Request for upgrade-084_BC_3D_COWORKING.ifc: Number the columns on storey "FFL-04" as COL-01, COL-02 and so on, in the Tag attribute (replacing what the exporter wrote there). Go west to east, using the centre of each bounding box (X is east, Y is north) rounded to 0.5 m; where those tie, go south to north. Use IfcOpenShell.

First a look at what the model holds.

```python
import ifcopenshell
import ifcopenshell.util.element
import ifcopenshell.util.placement

model = ifcopenshell.open("upgrade-084_BC_3D_COWORKING.ifc")
print(model.schema)
storey = next(s for s in model.by_type("IfcBuildingStorey") if s.Name == "FFL-04")
columns = [e for e in ifcopenshell.util.element.get_decomposition(storey) if e.is_a("IfcColumn")]
for e in sorted(columns, key=lambda e: e.id()):
    origin = ifcopenshell.util.placement.get_local_placement(e.ObjectPlacement)[:3, 3]
    print(e.id(), e.Tag, e.Name, origin.round(2) + 0.0, sep=" | ")
```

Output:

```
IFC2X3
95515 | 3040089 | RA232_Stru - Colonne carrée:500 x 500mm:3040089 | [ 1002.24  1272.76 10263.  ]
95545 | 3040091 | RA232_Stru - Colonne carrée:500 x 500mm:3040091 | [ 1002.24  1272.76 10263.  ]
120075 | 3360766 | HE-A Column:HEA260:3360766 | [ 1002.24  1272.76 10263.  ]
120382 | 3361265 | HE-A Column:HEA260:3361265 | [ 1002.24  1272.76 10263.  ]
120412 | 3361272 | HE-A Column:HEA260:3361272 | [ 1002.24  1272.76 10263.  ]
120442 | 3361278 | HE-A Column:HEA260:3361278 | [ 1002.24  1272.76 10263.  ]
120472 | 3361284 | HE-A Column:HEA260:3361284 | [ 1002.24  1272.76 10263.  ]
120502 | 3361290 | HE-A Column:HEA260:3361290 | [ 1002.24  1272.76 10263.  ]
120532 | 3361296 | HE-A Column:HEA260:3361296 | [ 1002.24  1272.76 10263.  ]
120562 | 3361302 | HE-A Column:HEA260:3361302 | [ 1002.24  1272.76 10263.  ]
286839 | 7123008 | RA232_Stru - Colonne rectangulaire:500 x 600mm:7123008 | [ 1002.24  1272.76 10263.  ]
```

```python
import ifcopenshell
import ifcopenshell.geom
import ifcopenshell.util.element
import ifcopenshell.util.shape

model = ifcopenshell.open("upgrade-084_BC_3D_COWORKING.ifc")
settings = ifcopenshell.geom.settings()
settings.set("use-world-coords", True)


def centre(element):
    shape = ifcopenshell.geom.create_shape(settings, element)
    return ifcopenshell.util.shape.get_bbox_centroid(shape.geometry)


storey = next(s for s in model.by_type("IfcBuildingStorey") if s.Name == "FFL-04")
columns = [e for e in ifcopenshell.util.element.get_decomposition(storey) if e.is_a("IfcColumn")]

# Insertion points can sit at a corner or the storey origin, so sort by the geometry (in metres).
centres = {e: centre(e) for e in columns}
columns.sort(key=lambda e: (round(centres[e][0] / 0.5), centres[e][1]))

for i, e in enumerate(columns, start=1):
    number = f"COL-{i:02d}"
    e.Tag = number
    print(e.id(), number)

model.write("upgrade-084_BC_3D_COWORKING_rev.ifc")
```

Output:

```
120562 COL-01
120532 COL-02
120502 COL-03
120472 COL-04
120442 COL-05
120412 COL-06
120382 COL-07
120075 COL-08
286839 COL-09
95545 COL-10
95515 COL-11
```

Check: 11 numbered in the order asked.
